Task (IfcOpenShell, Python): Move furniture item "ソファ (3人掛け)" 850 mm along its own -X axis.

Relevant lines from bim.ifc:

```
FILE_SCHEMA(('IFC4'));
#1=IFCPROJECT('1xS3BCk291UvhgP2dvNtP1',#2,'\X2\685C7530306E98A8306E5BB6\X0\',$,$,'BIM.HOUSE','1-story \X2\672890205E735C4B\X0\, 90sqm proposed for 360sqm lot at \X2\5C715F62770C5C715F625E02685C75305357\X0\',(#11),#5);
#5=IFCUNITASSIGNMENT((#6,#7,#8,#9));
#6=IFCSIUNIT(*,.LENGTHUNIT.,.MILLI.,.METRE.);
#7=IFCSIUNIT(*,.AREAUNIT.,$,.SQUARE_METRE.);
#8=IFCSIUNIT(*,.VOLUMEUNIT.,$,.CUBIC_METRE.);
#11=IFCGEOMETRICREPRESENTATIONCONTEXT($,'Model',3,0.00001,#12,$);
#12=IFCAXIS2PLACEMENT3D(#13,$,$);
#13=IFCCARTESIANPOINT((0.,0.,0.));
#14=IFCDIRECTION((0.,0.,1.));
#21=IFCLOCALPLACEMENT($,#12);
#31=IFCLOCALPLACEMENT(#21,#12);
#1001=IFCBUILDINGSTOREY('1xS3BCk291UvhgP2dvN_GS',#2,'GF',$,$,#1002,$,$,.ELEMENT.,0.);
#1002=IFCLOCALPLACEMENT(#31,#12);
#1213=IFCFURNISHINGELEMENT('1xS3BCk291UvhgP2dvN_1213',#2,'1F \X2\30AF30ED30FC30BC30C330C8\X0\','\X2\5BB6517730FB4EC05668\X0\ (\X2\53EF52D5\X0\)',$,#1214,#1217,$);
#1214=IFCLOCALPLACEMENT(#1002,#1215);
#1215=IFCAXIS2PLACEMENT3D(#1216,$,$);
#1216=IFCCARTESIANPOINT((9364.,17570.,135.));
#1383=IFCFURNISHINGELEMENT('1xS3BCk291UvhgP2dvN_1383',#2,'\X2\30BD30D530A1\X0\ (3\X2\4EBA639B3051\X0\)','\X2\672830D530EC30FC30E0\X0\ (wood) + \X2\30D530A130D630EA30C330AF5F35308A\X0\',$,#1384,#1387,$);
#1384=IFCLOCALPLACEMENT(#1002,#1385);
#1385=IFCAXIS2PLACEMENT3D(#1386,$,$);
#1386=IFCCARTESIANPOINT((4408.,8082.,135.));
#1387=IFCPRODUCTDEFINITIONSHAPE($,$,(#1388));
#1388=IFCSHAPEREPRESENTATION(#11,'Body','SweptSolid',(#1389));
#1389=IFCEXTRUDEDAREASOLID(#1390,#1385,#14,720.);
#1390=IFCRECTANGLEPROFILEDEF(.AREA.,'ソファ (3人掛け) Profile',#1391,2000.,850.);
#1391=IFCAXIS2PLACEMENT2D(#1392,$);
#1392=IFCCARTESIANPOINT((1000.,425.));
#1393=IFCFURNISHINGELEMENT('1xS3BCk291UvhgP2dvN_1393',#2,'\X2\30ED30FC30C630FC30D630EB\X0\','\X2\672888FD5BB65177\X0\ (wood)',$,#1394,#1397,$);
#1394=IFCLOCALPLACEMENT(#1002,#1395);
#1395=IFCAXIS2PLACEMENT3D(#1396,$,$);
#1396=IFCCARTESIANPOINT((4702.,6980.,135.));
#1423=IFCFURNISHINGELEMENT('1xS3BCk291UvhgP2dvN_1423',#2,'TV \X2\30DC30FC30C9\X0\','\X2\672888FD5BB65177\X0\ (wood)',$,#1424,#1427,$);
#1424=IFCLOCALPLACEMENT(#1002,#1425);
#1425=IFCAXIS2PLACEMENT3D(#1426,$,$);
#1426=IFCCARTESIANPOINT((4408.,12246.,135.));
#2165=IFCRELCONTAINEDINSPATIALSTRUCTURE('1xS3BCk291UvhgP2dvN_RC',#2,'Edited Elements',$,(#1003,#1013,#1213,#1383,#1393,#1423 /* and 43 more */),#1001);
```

```python
import ifcopenshell
import ifcopenshell.api.geometry
import ifcopenshell.util.placement

model = ifcopenshell.open("bim.ifc")

item = model.by_guid("1xS3BCk291UvhgP2dvN_1383")
matrix = ifcopenshell.util.placement.get_local_placement(item.ObjectPlacement)
matrix[:3, 3] -= matrix[:3, 0] * 850.0
ifcopenshell.api.geometry.edit_object_placement(model, product=item, matrix=matrix, is_si=False)

print(ifcopenshell.util.placement.get_local_placement(item.ObjectPlacement).round(3) + 0.0)

model.write("bim_v2.ifc")
```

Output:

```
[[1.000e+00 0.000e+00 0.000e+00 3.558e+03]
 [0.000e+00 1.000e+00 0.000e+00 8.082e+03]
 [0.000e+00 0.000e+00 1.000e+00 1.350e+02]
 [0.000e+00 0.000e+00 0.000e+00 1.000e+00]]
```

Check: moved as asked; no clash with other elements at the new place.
